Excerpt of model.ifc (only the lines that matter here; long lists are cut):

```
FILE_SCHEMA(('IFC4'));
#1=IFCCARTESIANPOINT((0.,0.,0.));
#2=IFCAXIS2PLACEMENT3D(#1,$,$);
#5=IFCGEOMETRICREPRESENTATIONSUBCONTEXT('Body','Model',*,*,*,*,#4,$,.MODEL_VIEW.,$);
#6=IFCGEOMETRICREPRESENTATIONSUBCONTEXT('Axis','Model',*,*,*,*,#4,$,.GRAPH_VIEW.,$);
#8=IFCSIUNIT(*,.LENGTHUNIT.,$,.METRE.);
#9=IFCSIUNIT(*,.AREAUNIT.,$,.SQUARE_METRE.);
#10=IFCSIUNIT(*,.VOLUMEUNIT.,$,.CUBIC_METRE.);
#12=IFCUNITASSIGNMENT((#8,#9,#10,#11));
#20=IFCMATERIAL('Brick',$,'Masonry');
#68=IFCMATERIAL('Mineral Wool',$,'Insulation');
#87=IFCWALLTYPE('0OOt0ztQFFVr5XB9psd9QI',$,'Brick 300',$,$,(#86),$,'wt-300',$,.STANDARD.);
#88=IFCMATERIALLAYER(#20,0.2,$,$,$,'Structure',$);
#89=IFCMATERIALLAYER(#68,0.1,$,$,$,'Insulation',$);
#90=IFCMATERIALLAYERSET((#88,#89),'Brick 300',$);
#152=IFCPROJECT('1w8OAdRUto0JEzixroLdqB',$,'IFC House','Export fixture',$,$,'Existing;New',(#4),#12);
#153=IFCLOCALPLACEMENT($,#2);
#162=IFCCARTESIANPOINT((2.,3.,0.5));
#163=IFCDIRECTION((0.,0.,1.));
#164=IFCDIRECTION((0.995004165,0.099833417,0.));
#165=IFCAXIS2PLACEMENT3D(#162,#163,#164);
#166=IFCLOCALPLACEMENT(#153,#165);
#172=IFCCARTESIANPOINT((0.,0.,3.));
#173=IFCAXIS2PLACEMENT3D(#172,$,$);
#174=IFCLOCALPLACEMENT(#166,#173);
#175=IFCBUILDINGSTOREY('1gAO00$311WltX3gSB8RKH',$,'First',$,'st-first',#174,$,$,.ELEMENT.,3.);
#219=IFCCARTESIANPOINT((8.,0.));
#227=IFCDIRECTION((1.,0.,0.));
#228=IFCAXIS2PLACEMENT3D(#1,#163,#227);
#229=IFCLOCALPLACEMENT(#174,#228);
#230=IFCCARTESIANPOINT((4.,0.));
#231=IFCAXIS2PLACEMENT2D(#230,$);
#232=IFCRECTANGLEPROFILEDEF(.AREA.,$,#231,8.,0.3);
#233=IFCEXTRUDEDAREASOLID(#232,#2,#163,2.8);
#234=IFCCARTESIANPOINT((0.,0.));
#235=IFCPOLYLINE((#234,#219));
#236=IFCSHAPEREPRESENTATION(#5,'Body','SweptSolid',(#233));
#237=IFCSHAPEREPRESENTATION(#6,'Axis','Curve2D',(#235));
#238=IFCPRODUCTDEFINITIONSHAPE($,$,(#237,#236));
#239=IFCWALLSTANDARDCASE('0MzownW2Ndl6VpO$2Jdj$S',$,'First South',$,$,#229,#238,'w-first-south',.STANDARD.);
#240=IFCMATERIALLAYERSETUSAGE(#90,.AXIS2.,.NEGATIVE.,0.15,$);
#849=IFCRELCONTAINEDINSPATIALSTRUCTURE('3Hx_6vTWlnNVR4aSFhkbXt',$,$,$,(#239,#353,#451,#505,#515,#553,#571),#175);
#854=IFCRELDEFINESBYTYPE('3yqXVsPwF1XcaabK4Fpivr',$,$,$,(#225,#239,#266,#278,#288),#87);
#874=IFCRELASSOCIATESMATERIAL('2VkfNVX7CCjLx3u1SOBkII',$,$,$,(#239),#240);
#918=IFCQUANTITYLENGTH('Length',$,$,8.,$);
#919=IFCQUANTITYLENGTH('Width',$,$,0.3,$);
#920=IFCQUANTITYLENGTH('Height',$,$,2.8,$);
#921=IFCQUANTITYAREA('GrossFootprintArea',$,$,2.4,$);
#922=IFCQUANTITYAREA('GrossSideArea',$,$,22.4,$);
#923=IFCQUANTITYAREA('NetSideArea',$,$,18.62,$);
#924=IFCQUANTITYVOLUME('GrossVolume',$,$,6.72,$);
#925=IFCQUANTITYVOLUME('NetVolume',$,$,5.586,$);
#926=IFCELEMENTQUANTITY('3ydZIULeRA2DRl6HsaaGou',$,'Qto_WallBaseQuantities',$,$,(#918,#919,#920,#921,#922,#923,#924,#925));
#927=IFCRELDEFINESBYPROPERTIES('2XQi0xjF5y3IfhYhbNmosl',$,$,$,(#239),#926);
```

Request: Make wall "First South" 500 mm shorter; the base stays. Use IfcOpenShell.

```python
import ifcopenshell
import ifcopenshell.api.pset
import ifcopenshell.geom
import ifcopenshell.util.element
import ifcopenshell.util.representation
import ifcopenshell.util.shape
import ifcopenshell.util.unit

model = ifcopenshell.open("model.ifc")
unit_scale = ifcopenshell.util.unit.calculate_unit_scale(model)
area_scale = ifcopenshell.util.unit.calculate_unit_scale(model, "AREAUNIT")
volume_scale = ifcopenshell.util.unit.calculate_unit_scale(model, "VOLUMEUNIT")
settings = ifcopenshell.geom.settings()


def volume(element):
    """Net volume in cubic metres, openings subtracted."""
    shape = ifcopenshell.geom.create_shape(settings, element)
    return ifcopenshell.util.shape.get_volume(shape.geometry)


wall = model.by_guid("0MzownW2Ndl6VpO$2Jdj$S")
before = volume(wall)

body = ifcopenshell.util.representation.get_representation(wall, "Model", "Body")
solid = body.Items[0]
old_height = solid.Depth
solid.Depth -= 0.5 / unit_scale
after = volume(wall)
thickness = 0.3  # wall thickness in metres

# Update the stored height, areas and volumes.
qto = model.by_id(ifcopenshell.util.element.get_pset(wall, "Qto_WallBaseQuantities", should_inherit=False)["id"])
ifcopenshell.api.pset.edit_qto(model, qto=qto, properties={
    "Height": solid.Depth,
    "GrossSideArea": ifcopenshell.util.element.get_pset(wall, "Qto_WallBaseQuantities", "GrossSideArea") * solid.Depth / old_height,
    "NetSideArea": after / thickness / area_scale,
    "GrossVolume": ifcopenshell.util.element.get_pset(wall, "Qto_WallBaseQuantities", "GrossVolume") * solid.Depth / old_height,
    "NetVolume": after / volume_scale,
})

print(f"height {old_height:g} -> {solid.Depth:g}, volume {before:.3f} -> {after:.3f} m3")

model.write("model_rev.ifc")
```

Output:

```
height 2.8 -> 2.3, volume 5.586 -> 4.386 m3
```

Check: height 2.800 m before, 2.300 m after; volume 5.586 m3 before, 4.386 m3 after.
